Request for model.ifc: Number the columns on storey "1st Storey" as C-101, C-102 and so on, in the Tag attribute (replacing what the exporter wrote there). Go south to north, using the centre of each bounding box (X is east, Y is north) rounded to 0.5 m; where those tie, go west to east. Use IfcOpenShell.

First a look at what the model holds.

```python
import ifcopenshell
import ifcopenshell.util.element
import ifcopenshell.util.placement

model = ifcopenshell.open("model.ifc")
print(model.schema)
storey = next(s for s in model.by_type("IfcBuildingStorey") if s.Name == "1st Storey")
columns = [e for e in ifcopenshell.util.element.get_decomposition(storey) if e.is_a("IfcColumn")]
for e in sorted(columns, key=lambda e: e.id()):
    origin = ifcopenshell.util.placement.get_local_placement(e.ObjectPlacement)[:3, 3]
    print(e.id(), e.Tag, e.Name, origin.round(2) + 0.0, sep=" | ")
```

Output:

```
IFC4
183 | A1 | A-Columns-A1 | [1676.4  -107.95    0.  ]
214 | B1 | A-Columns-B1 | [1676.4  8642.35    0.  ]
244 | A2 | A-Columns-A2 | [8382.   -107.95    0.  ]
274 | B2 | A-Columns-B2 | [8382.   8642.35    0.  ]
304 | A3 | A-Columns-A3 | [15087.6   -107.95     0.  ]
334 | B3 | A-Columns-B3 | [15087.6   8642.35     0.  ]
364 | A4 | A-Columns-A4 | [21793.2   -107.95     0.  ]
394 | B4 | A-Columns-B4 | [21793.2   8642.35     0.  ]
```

```python
import ifcopenshell
import ifcopenshell.geom
import ifcopenshell.util.element
import ifcopenshell.util.shape

model = ifcopenshell.open("model.ifc")
settings = ifcopenshell.geom.settings()
settings.set("use-world-coords", True)


def centre(element):
    shape = ifcopenshell.geom.create_shape(settings, element)
    return ifcopenshell.util.shape.get_bbox_centroid(shape.geometry)


storey = next(s for s in model.by_type("IfcBuildingStorey") if s.Name == "1st Storey")
columns = [e for e in ifcopenshell.util.element.get_decomposition(storey) if e.is_a("IfcColumn")]

# Insertion points can sit at a corner or the storey origin, so sort by the geometry (in metres).
centres = {e: centre(e) for e in columns}
columns.sort(key=lambda e: (round(centres[e][1] / 0.5), centres[e][0]))

for i, e in enumerate(columns, start=1):
    number = f"C-1{i:02d}"
    e.Tag = number
    print(e.id(), number)

model.write("model-out.ifc")
```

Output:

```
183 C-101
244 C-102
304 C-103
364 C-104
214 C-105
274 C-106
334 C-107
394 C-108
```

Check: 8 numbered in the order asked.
